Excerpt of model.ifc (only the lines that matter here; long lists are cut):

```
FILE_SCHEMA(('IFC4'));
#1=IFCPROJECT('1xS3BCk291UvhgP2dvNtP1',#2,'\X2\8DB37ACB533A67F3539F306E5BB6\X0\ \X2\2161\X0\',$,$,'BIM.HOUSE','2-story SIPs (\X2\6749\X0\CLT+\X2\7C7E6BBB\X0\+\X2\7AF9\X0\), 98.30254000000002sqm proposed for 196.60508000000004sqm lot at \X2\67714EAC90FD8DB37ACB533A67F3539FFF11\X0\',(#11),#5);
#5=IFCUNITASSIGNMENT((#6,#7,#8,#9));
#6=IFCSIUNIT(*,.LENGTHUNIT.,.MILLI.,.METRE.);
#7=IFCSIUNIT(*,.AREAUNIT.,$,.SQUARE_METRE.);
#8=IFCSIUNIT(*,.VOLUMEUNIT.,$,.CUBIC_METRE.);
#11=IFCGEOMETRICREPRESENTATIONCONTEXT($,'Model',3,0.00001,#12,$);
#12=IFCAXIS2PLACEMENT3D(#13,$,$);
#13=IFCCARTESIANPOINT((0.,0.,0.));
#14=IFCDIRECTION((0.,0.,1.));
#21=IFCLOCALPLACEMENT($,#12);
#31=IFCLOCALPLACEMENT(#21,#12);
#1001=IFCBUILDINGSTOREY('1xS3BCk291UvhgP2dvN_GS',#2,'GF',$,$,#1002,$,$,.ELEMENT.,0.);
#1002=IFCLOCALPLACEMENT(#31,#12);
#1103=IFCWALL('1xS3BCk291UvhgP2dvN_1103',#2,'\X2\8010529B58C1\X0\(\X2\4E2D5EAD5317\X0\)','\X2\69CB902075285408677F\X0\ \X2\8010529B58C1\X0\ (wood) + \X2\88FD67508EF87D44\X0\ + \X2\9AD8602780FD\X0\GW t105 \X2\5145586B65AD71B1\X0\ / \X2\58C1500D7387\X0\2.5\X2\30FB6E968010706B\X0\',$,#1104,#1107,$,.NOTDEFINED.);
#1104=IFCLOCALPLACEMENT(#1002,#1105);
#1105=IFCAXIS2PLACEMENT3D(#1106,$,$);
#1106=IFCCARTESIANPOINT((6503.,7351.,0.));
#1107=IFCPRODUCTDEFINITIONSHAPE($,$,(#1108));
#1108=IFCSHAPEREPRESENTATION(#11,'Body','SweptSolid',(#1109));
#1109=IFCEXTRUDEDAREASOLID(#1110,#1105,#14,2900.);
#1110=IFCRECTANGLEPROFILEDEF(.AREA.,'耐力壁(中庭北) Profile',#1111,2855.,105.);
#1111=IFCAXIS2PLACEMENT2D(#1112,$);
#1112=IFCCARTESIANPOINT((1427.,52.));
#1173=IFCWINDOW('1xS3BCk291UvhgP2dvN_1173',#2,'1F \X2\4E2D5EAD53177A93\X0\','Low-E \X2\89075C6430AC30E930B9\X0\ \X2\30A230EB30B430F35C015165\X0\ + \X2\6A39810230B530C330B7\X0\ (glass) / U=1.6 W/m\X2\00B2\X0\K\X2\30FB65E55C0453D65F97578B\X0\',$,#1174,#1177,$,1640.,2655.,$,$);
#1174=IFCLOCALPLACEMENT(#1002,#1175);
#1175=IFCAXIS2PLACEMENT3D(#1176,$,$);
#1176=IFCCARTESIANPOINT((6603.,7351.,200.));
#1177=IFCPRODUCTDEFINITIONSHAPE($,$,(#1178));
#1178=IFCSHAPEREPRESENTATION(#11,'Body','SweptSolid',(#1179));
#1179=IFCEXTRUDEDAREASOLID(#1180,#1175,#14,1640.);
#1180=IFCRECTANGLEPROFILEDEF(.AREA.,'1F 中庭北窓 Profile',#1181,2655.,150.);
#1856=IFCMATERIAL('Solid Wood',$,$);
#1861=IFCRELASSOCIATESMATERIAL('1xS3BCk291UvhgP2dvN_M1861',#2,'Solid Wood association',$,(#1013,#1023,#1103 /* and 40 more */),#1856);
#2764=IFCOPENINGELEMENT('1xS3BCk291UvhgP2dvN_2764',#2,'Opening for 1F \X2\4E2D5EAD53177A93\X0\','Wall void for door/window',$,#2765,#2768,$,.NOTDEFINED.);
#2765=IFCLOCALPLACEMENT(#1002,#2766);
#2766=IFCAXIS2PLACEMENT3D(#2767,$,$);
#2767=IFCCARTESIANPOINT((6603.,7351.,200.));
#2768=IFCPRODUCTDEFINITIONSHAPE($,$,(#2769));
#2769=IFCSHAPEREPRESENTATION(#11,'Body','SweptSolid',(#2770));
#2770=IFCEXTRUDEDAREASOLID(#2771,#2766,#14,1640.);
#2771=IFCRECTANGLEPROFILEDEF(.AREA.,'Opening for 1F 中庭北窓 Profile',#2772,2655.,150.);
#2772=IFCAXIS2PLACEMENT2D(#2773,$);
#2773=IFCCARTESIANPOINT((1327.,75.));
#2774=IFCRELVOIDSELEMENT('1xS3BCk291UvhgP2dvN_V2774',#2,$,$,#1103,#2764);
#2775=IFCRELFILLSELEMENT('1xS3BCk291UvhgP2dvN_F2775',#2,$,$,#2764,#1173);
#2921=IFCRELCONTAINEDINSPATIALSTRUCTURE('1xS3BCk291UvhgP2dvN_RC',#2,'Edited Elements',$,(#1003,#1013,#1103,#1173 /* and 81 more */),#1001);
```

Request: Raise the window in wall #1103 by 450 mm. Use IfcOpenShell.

```python
import numpy as np
import ifcopenshell
import ifcopenshell.api.geometry
import ifcopenshell.util.placement
import ifcopenshell.util.unit

model = ifcopenshell.open("model.ifc")
unit_scale = ifcopenshell.util.unit.calculate_unit_scale(model)

window = model.by_id(1173)
opening = window.FillsVoids[0].RelatingOpeningElement
dz = 450.0

shift = np.array([0.0, 0.0, dz])
# The window is not placed relative to its opening, so move both.
for product in (opening, window):
    matrix = ifcopenshell.util.placement.get_local_placement(product.ObjectPlacement)
    matrix[:3, 3] += shift
    ifcopenshell.api.geometry.edit_object_placement(model, product=product, matrix=matrix, is_si=False)

print(f"moved by {dz * unit_scale:+.3f} m")

model.write("model-out.ifc")
```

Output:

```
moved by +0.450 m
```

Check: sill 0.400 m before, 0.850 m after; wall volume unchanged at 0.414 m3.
